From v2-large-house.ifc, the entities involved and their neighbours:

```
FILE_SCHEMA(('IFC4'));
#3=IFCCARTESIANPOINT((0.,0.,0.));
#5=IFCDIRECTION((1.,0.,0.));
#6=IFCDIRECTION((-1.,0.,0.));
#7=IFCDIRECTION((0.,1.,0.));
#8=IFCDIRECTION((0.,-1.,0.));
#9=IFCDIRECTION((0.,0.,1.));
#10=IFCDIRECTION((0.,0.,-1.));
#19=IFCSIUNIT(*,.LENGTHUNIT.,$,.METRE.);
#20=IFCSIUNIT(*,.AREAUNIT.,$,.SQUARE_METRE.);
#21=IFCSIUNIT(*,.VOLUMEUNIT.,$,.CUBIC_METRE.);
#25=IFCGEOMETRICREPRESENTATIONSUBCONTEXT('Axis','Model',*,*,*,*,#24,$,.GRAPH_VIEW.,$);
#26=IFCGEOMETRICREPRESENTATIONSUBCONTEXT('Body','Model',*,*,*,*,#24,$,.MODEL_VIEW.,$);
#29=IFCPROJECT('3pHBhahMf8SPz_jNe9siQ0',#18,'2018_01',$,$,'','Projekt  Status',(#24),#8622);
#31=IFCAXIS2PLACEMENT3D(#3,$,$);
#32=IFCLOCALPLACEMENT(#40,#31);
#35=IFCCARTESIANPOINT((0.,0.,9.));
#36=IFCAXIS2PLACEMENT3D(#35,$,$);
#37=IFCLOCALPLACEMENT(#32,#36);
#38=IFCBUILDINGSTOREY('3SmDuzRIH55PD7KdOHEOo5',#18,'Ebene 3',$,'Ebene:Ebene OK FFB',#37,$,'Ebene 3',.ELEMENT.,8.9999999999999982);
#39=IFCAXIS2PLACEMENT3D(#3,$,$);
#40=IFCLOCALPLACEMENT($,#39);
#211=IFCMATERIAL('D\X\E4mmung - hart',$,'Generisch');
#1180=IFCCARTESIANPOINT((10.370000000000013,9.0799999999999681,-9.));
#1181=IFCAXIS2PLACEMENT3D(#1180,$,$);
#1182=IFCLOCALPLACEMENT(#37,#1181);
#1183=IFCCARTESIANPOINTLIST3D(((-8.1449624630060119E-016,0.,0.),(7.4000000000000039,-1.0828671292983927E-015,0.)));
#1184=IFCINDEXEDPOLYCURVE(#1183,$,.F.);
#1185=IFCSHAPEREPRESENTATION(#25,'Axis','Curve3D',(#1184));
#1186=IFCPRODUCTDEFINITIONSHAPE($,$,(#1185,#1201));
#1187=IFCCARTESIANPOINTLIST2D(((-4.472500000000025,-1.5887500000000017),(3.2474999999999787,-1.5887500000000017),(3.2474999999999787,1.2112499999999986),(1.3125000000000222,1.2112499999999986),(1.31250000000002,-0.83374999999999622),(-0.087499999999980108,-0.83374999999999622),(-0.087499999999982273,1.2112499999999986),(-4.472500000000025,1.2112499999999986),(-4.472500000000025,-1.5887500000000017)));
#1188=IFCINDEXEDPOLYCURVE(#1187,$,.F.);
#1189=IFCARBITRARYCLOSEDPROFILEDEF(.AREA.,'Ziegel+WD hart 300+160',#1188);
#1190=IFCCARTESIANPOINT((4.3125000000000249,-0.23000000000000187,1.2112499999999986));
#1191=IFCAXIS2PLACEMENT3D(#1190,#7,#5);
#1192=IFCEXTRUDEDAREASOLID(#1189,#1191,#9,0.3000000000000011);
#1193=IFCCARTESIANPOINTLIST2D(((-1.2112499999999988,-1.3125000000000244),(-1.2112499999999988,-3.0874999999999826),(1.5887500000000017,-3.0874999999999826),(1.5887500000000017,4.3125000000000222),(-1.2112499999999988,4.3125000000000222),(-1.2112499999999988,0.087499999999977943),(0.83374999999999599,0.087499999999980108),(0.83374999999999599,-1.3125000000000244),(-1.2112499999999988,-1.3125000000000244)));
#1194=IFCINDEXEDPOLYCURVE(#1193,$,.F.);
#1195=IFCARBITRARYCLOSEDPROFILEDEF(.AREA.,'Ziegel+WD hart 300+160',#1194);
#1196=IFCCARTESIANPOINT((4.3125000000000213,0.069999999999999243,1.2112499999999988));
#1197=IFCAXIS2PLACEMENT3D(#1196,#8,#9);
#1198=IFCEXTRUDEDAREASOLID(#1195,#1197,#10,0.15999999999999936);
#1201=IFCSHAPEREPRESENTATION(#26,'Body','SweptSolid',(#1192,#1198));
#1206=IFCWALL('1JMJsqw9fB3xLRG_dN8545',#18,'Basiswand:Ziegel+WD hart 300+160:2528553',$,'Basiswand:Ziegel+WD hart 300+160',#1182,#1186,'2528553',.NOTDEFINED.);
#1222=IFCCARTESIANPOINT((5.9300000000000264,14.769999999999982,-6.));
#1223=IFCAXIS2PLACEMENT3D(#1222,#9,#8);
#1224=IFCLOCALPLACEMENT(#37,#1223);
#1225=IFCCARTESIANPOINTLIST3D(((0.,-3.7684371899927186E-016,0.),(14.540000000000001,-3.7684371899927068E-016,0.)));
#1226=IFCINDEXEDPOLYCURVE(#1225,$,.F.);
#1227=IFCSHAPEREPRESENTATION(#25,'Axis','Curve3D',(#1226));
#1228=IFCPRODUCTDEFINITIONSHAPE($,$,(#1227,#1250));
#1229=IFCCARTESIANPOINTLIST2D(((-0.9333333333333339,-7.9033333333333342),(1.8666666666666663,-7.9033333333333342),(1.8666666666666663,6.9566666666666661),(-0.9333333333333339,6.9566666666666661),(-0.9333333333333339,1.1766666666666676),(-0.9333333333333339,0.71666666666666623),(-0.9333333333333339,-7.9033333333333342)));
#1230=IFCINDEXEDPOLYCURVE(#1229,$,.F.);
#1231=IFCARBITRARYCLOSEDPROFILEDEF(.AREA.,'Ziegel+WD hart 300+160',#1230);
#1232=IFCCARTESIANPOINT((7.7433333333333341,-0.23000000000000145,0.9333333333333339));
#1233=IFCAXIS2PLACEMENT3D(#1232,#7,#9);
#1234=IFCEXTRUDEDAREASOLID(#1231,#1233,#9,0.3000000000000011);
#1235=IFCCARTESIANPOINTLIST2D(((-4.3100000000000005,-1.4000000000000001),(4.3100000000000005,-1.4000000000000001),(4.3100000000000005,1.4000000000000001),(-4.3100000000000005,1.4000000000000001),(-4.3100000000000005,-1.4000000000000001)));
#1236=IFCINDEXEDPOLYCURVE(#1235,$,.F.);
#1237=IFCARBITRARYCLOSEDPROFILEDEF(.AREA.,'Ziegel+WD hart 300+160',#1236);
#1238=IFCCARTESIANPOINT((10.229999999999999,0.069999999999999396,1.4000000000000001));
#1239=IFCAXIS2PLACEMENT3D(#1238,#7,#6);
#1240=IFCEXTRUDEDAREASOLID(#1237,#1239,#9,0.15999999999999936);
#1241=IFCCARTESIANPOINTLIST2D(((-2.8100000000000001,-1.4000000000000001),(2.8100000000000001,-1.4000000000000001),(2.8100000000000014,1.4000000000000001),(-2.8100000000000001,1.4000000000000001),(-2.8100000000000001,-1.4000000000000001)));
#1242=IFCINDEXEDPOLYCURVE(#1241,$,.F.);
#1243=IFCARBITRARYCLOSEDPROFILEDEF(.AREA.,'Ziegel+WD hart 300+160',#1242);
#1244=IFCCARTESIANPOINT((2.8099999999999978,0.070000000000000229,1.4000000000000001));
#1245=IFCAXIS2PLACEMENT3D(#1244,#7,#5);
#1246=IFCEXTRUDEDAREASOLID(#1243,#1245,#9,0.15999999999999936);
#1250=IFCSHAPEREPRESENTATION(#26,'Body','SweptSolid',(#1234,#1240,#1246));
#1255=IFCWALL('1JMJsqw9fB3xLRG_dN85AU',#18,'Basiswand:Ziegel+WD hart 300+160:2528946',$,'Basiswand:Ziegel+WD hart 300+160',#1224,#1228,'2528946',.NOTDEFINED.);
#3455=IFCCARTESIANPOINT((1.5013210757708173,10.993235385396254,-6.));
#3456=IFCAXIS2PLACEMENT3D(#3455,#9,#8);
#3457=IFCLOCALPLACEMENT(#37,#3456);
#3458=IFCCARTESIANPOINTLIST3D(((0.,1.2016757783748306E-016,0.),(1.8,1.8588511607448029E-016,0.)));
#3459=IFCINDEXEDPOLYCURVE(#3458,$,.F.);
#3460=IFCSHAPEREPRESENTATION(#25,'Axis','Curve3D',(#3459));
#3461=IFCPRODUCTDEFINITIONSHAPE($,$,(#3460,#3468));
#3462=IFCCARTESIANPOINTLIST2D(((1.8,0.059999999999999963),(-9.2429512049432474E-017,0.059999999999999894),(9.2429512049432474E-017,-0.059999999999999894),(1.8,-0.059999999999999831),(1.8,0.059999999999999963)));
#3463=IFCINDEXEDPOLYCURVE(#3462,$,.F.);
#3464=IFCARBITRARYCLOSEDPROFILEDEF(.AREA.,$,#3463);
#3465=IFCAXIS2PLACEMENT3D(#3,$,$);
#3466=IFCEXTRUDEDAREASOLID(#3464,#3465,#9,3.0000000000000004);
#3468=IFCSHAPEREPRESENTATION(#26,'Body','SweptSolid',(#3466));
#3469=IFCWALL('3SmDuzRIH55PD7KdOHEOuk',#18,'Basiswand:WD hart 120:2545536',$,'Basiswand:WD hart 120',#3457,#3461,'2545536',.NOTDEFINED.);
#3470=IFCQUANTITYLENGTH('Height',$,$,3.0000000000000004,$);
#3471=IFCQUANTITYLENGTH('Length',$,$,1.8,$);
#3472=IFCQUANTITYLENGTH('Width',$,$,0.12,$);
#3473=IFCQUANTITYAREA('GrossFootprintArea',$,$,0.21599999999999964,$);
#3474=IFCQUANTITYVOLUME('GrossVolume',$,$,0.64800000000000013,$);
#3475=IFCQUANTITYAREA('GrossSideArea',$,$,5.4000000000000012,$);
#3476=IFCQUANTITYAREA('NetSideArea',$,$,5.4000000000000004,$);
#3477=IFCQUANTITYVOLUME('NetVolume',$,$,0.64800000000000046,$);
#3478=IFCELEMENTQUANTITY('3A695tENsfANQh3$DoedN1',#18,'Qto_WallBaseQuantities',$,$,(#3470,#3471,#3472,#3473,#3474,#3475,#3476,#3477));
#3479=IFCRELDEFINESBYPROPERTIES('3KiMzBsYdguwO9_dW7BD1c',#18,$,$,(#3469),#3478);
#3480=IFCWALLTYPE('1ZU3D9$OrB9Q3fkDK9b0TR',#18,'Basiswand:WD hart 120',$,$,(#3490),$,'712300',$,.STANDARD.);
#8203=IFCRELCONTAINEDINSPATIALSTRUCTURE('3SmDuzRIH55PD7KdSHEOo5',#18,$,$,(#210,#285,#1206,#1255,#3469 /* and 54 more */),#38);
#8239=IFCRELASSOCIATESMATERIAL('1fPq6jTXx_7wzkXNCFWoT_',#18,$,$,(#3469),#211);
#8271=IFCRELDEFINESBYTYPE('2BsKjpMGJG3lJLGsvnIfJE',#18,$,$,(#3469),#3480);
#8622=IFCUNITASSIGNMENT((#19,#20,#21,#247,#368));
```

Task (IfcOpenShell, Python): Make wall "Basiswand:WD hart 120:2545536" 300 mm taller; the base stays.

```python
import ifcopenshell
import ifcopenshell.api.pset
import ifcopenshell.geom
import ifcopenshell.util.element
import ifcopenshell.util.representation
import ifcopenshell.util.shape
import ifcopenshell.util.unit

model = ifcopenshell.open("v2-large-house.ifc")
unit_scale = ifcopenshell.util.unit.calculate_unit_scale(model)
area_scale = ifcopenshell.util.unit.calculate_unit_scale(model, "AREAUNIT")
volume_scale = ifcopenshell.util.unit.calculate_unit_scale(model, "VOLUMEUNIT")
settings = ifcopenshell.geom.settings()


def volume(element):
    """Net volume in cubic metres, openings subtracted."""
    shape = ifcopenshell.geom.create_shape(settings, element)
    return ifcopenshell.util.shape.get_volume(shape.geometry)


wall = model.by_guid("3SmDuzRIH55PD7KdOHEOuk")
before = volume(wall)

body = ifcopenshell.util.representation.get_representation(wall, "Model", "Body")
solid = body.Items[0]
old_height = solid.Depth
solid.Depth += 0.3 / unit_scale
after = volume(wall)
thickness = 0.12  # wall thickness in metres

# Update the stored height, areas and volumes.
qto = model.by_id(ifcopenshell.util.element.get_pset(wall, "Qto_WallBaseQuantities", should_inherit=False)["id"])
ifcopenshell.api.pset.edit_qto(model, qto=qto, properties={
    "Height": solid.Depth,
    "GrossVolume": ifcopenshell.util.element.get_pset(wall, "Qto_WallBaseQuantities", "GrossVolume") * solid.Depth / old_height,
    "GrossSideArea": ifcopenshell.util.element.get_pset(wall, "Qto_WallBaseQuantities", "GrossSideArea") * solid.Depth / old_height,
    "NetSideArea": after / thickness / area_scale,
    "NetVolume": after / volume_scale,
})

print(f"height {old_height:g} -> {solid.Depth:g}, volume {before:.3f} -> {after:.3f} m3")

model.write("v2-large-house-out.ifc")
```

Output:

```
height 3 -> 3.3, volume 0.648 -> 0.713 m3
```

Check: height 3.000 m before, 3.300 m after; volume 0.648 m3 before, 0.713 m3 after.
